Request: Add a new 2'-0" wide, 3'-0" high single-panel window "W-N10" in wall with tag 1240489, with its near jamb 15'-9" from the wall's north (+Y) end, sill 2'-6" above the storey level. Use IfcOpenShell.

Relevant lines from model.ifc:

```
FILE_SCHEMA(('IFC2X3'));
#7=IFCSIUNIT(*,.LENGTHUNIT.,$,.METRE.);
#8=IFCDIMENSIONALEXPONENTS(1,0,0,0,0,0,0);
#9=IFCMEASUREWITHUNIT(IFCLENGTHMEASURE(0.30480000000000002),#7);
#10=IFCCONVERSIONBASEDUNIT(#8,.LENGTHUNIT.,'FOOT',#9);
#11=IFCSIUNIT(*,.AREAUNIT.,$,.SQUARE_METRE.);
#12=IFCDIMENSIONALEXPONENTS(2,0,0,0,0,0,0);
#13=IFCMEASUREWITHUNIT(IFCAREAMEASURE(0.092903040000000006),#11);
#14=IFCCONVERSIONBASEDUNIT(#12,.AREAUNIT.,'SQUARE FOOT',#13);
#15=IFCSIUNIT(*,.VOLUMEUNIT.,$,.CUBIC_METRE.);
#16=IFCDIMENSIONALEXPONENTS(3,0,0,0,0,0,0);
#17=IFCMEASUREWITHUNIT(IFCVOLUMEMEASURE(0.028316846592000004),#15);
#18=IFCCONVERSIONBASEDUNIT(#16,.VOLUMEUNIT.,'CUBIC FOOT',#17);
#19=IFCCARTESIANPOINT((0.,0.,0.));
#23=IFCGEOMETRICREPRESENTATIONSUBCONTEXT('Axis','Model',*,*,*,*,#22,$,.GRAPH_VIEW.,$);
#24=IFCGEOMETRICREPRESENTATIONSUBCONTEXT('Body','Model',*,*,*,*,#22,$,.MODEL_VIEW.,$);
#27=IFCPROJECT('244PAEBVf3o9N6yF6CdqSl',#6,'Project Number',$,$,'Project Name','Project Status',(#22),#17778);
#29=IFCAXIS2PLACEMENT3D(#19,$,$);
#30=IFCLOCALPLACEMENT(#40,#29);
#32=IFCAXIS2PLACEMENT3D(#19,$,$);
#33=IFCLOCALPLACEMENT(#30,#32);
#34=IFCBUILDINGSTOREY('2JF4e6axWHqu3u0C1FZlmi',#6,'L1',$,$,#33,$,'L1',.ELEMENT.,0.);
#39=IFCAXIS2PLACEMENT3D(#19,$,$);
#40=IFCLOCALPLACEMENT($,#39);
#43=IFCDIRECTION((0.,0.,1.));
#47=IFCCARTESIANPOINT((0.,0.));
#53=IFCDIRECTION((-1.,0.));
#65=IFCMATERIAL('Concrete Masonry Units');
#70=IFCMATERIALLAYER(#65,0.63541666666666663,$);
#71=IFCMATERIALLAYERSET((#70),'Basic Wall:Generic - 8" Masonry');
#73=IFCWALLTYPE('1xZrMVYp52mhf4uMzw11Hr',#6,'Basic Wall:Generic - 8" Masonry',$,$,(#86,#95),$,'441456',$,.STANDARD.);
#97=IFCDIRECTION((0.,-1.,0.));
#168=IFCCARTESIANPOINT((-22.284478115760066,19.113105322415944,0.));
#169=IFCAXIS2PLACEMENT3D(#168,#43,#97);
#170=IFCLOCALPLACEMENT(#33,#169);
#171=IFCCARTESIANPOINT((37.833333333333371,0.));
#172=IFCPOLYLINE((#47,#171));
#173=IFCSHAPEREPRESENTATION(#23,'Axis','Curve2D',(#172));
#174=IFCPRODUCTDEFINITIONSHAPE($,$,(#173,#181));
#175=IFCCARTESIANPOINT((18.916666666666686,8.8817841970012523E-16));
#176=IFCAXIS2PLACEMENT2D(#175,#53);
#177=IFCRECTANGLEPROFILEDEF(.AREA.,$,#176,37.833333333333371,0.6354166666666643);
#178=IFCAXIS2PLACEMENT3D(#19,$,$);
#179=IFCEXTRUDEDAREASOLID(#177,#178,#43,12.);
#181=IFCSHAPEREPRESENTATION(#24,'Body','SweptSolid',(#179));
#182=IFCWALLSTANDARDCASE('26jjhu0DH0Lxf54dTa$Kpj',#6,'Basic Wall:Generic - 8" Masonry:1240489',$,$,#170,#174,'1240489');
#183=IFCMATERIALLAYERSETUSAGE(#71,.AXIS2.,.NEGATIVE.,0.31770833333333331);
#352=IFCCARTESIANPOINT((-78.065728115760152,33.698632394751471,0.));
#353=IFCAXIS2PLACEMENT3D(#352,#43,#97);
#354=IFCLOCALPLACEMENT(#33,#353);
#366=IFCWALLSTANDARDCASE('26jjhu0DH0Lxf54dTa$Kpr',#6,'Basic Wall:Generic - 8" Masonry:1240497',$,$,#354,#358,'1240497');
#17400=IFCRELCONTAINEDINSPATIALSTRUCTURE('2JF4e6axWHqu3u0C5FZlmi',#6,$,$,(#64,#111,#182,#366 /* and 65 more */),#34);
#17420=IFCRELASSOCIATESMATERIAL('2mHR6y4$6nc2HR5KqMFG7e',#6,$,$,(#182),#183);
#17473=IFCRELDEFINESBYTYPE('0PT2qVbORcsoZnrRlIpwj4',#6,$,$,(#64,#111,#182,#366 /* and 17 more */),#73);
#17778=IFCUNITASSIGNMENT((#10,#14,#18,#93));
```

```python
import numpy as np
import ifcopenshell
import ifcopenshell.api.feature
import ifcopenshell.api.geometry
import ifcopenshell.api.root
import ifcopenshell.api.spatial
import ifcopenshell.api.type
import ifcopenshell.geom
import ifcopenshell.util.element
import ifcopenshell.util.placement
import ifcopenshell.util.representation
import ifcopenshell.util.shape
import ifcopenshell.util.unit

model = ifcopenshell.open("model.ifc")
unit_scale = ifcopenshell.util.unit.calculate_unit_scale(model)
settings = ifcopenshell.geom.settings()


def volume(element):
    """Net volume in cubic metres, openings subtracted."""
    shape = ifcopenshell.geom.create_shape(settings, element)
    return ifcopenshell.util.shape.get_volume(shape.geometry)


wall = model.by_guid("26jjhu0DH0Lxf54dTa$Kpj")
storey = ifcopenshell.util.element.get_container(wall, ifc_class="IfcBuildingStorey")
context = ifcopenshell.util.representation.get_context(model, "Model", "Body", "MODEL_VIEW")
before = volume(wall)

width, height, from_end, sill = 0.6096, 0.9144, 4.8006, 0.762  # metres

# The wall runs along its own X axis, and the end named is its -X end.
wall_shape = ifcopenshell.geom.create_shape(settings, wall)
x, y, z = ifcopenshell.util.shape.get_vertices(wall_shape.geometry).T
start = x.min() + from_end
face, thickness = float(y.min()), float(y.max() - y.min())
wall_matrix = ifcopenshell.util.placement.get_local_placement(wall.ObjectPlacement)
level = ifcopenshell.util.placement.get_local_placement(storey.ObjectPlacement)[2, 3]


def in_wall(x, y):
    """Placement at x, y metres in the wall's axes, at sill height."""
    matrix = wall_matrix.copy()
    matrix[:, 3] = wall_matrix @ np.array([x / unit_scale, y / unit_scale, 0.0, 1.0])
    matrix[2, 3] = level + sill / unit_scale
    return matrix


# Opening: a box that overshoots both wall faces by 50 mm.
opening = ifcopenshell.api.root.create_entity(model, ifc_class="IfcOpeningElement")
box = ifcopenshell.api.geometry.add_wall_representation(
    model, context=context, length=width, height=height, thickness=thickness + 0.1
)
ifcopenshell.api.geometry.assign_representation(model, product=opening, representation=box)
ifcopenshell.api.geometry.edit_object_placement(model, product=opening, matrix=in_wall(start, face - 0.05), is_si=False)
ifcopenshell.api.feature.add_feature(model, feature=opening, element=wall)

window = ifcopenshell.api.root.create_entity(model, ifc_class="IfcWindow", name="W-N10")
window.OverallWidth, window.OverallHeight = width / unit_scale, height / unit_scale
body = ifcopenshell.api.geometry.add_window_representation(
    model,
    context=context,
    overall_width=window.OverallWidth,
    overall_height=window.OverallHeight,
    partition_type="SINGLE_PANEL",
)
ifcopenshell.api.geometry.assign_representation(model, product=window, representation=body)
ifcopenshell.api.spatial.assign_container(model, products=[window], relating_structure=storey)
fills = ifcopenshell.api.feature.add_filling(model, opening=opening, element=window)
fills.OwnerHistory = window.OwnerHistory  # required in IFC2X3

# IFC2X3 keeps the operation on the window style.
style = ifcopenshell.api.root.create_entity(model, ifc_class="IfcWindowStyle", name="W-N10")
style.OperationType, style.ConstructionType = "SINGLE_PANEL", "NOTDEFINED"
style.ParameterTakesPrecedence = style.Sizeable = False
ifcopenshell.api.type.assign_type(model, related_objects=[window], relating_type=style)

# Centre the window in the wall's thickness.
ifcopenshell.api.geometry.edit_object_placement(model, product=window, matrix=in_wall(start, face), is_si=False)
window_shape = ifcopenshell.geom.create_shape(settings, window)
depth = ifcopenshell.util.shape.get_vertices(window_shape.geometry)[:, 1]
offset = face + thickness / 2 - (depth.min() + depth.max()) / 2
ifcopenshell.api.geometry.edit_object_placement(model, product=window, matrix=in_wall(start, offset), is_si=False)

after = volume(wall)

print(f"wall volume {before:.3f} -> {after:.3f} m3")

model.write("model_edited.ifc")
```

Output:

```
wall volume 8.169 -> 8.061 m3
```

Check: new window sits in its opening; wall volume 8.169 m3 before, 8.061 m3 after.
